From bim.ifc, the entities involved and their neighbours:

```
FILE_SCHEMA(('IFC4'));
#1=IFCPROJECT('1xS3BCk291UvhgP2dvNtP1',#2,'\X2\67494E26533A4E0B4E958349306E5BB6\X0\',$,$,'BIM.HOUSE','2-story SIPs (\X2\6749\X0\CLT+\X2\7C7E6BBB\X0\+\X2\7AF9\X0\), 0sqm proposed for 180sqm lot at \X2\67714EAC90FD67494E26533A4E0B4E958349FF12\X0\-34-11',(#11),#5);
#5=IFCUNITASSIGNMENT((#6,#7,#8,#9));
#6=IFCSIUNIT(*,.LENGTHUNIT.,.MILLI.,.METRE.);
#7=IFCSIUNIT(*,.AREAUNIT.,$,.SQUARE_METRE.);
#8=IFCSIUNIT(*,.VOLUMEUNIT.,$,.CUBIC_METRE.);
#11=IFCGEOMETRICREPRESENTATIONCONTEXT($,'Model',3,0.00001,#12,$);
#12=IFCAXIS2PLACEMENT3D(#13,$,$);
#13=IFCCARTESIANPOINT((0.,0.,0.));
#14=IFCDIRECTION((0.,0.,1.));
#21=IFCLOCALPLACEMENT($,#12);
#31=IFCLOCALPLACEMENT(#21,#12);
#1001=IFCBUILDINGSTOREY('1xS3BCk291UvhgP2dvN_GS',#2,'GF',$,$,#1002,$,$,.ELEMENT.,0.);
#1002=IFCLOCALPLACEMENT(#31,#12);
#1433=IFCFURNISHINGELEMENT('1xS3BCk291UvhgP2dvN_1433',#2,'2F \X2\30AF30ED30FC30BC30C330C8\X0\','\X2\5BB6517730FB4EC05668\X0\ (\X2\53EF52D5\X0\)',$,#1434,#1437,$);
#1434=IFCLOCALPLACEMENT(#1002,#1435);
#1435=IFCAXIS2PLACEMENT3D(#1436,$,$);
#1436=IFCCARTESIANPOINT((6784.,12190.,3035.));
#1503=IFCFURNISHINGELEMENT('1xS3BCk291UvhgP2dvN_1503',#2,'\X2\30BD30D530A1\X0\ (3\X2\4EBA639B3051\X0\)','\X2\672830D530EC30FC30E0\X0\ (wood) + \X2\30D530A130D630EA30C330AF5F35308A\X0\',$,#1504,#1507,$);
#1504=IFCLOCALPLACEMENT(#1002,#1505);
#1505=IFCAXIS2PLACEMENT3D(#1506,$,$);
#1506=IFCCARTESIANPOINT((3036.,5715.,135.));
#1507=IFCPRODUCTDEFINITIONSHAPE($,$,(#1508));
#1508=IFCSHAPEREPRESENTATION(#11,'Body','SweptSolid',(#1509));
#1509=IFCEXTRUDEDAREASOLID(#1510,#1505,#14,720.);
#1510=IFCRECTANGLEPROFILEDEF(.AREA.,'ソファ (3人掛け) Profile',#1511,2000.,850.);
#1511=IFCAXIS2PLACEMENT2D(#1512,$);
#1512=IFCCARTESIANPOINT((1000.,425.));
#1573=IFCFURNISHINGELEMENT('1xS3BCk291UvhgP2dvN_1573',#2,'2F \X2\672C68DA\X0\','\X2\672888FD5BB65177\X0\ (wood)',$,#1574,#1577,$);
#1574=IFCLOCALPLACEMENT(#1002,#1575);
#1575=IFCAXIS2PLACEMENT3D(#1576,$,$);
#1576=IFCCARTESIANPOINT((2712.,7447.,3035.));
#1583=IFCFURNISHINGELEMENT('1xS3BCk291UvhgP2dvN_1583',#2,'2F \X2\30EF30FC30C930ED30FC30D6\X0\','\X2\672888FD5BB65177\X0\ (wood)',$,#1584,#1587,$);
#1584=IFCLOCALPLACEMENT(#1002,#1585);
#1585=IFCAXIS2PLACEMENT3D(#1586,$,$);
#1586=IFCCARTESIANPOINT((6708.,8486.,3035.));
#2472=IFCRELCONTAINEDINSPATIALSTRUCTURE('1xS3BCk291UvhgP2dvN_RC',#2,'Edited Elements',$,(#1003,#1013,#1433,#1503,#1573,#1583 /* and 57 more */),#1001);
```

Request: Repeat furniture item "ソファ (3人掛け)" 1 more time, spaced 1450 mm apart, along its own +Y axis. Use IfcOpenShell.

```python
import ifcopenshell
import ifcopenshell.api.geometry
import ifcopenshell.api.root
import ifcopenshell.util.element
import ifcopenshell.util.placement

model = ifcopenshell.open("bim.ifc")


def reuse_history(source, copy):
    """copy_class also copies each property set's owner history, people and application; keep the originals."""
    for rel in copy.IsDefinedBy:
        if rel.is_a("IfcRelDefinesByProperties") and (history := rel.RelatingPropertyDefinition.OwnerHistory):
            rel.RelatingPropertyDefinition.OwnerHistory = source.OwnerHistory
            ifcopenshell.util.element.remove_deep2(model, history)


source = model.by_guid("1xS3BCk291UvhgP2dvN_1503")
base = ifcopenshell.util.placement.get_local_placement(source.ObjectPlacement)
step = base[:3, 1] * 1450.0

for i in range(1, 2):
    copy = ifcopenshell.api.root.copy_class(model, product=source)
    copy.Representation = ifcopenshell.util.element.copy_deep(
        model, source.Representation, exclude=["IfcGeometricRepresentationContext", "IfcRepresentationMap"]
    )
    reuse_history(source, copy)
    matrix = base.copy()
    matrix[:3, 3] += i * step
    print("added at", matrix[:3, 3].round(3) + 0.0)
    ifcopenshell.api.geometry.edit_object_placement(model, product=copy, matrix=matrix, is_si=False)

model.write("bim_v2.ifc")
```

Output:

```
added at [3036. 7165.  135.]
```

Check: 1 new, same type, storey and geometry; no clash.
